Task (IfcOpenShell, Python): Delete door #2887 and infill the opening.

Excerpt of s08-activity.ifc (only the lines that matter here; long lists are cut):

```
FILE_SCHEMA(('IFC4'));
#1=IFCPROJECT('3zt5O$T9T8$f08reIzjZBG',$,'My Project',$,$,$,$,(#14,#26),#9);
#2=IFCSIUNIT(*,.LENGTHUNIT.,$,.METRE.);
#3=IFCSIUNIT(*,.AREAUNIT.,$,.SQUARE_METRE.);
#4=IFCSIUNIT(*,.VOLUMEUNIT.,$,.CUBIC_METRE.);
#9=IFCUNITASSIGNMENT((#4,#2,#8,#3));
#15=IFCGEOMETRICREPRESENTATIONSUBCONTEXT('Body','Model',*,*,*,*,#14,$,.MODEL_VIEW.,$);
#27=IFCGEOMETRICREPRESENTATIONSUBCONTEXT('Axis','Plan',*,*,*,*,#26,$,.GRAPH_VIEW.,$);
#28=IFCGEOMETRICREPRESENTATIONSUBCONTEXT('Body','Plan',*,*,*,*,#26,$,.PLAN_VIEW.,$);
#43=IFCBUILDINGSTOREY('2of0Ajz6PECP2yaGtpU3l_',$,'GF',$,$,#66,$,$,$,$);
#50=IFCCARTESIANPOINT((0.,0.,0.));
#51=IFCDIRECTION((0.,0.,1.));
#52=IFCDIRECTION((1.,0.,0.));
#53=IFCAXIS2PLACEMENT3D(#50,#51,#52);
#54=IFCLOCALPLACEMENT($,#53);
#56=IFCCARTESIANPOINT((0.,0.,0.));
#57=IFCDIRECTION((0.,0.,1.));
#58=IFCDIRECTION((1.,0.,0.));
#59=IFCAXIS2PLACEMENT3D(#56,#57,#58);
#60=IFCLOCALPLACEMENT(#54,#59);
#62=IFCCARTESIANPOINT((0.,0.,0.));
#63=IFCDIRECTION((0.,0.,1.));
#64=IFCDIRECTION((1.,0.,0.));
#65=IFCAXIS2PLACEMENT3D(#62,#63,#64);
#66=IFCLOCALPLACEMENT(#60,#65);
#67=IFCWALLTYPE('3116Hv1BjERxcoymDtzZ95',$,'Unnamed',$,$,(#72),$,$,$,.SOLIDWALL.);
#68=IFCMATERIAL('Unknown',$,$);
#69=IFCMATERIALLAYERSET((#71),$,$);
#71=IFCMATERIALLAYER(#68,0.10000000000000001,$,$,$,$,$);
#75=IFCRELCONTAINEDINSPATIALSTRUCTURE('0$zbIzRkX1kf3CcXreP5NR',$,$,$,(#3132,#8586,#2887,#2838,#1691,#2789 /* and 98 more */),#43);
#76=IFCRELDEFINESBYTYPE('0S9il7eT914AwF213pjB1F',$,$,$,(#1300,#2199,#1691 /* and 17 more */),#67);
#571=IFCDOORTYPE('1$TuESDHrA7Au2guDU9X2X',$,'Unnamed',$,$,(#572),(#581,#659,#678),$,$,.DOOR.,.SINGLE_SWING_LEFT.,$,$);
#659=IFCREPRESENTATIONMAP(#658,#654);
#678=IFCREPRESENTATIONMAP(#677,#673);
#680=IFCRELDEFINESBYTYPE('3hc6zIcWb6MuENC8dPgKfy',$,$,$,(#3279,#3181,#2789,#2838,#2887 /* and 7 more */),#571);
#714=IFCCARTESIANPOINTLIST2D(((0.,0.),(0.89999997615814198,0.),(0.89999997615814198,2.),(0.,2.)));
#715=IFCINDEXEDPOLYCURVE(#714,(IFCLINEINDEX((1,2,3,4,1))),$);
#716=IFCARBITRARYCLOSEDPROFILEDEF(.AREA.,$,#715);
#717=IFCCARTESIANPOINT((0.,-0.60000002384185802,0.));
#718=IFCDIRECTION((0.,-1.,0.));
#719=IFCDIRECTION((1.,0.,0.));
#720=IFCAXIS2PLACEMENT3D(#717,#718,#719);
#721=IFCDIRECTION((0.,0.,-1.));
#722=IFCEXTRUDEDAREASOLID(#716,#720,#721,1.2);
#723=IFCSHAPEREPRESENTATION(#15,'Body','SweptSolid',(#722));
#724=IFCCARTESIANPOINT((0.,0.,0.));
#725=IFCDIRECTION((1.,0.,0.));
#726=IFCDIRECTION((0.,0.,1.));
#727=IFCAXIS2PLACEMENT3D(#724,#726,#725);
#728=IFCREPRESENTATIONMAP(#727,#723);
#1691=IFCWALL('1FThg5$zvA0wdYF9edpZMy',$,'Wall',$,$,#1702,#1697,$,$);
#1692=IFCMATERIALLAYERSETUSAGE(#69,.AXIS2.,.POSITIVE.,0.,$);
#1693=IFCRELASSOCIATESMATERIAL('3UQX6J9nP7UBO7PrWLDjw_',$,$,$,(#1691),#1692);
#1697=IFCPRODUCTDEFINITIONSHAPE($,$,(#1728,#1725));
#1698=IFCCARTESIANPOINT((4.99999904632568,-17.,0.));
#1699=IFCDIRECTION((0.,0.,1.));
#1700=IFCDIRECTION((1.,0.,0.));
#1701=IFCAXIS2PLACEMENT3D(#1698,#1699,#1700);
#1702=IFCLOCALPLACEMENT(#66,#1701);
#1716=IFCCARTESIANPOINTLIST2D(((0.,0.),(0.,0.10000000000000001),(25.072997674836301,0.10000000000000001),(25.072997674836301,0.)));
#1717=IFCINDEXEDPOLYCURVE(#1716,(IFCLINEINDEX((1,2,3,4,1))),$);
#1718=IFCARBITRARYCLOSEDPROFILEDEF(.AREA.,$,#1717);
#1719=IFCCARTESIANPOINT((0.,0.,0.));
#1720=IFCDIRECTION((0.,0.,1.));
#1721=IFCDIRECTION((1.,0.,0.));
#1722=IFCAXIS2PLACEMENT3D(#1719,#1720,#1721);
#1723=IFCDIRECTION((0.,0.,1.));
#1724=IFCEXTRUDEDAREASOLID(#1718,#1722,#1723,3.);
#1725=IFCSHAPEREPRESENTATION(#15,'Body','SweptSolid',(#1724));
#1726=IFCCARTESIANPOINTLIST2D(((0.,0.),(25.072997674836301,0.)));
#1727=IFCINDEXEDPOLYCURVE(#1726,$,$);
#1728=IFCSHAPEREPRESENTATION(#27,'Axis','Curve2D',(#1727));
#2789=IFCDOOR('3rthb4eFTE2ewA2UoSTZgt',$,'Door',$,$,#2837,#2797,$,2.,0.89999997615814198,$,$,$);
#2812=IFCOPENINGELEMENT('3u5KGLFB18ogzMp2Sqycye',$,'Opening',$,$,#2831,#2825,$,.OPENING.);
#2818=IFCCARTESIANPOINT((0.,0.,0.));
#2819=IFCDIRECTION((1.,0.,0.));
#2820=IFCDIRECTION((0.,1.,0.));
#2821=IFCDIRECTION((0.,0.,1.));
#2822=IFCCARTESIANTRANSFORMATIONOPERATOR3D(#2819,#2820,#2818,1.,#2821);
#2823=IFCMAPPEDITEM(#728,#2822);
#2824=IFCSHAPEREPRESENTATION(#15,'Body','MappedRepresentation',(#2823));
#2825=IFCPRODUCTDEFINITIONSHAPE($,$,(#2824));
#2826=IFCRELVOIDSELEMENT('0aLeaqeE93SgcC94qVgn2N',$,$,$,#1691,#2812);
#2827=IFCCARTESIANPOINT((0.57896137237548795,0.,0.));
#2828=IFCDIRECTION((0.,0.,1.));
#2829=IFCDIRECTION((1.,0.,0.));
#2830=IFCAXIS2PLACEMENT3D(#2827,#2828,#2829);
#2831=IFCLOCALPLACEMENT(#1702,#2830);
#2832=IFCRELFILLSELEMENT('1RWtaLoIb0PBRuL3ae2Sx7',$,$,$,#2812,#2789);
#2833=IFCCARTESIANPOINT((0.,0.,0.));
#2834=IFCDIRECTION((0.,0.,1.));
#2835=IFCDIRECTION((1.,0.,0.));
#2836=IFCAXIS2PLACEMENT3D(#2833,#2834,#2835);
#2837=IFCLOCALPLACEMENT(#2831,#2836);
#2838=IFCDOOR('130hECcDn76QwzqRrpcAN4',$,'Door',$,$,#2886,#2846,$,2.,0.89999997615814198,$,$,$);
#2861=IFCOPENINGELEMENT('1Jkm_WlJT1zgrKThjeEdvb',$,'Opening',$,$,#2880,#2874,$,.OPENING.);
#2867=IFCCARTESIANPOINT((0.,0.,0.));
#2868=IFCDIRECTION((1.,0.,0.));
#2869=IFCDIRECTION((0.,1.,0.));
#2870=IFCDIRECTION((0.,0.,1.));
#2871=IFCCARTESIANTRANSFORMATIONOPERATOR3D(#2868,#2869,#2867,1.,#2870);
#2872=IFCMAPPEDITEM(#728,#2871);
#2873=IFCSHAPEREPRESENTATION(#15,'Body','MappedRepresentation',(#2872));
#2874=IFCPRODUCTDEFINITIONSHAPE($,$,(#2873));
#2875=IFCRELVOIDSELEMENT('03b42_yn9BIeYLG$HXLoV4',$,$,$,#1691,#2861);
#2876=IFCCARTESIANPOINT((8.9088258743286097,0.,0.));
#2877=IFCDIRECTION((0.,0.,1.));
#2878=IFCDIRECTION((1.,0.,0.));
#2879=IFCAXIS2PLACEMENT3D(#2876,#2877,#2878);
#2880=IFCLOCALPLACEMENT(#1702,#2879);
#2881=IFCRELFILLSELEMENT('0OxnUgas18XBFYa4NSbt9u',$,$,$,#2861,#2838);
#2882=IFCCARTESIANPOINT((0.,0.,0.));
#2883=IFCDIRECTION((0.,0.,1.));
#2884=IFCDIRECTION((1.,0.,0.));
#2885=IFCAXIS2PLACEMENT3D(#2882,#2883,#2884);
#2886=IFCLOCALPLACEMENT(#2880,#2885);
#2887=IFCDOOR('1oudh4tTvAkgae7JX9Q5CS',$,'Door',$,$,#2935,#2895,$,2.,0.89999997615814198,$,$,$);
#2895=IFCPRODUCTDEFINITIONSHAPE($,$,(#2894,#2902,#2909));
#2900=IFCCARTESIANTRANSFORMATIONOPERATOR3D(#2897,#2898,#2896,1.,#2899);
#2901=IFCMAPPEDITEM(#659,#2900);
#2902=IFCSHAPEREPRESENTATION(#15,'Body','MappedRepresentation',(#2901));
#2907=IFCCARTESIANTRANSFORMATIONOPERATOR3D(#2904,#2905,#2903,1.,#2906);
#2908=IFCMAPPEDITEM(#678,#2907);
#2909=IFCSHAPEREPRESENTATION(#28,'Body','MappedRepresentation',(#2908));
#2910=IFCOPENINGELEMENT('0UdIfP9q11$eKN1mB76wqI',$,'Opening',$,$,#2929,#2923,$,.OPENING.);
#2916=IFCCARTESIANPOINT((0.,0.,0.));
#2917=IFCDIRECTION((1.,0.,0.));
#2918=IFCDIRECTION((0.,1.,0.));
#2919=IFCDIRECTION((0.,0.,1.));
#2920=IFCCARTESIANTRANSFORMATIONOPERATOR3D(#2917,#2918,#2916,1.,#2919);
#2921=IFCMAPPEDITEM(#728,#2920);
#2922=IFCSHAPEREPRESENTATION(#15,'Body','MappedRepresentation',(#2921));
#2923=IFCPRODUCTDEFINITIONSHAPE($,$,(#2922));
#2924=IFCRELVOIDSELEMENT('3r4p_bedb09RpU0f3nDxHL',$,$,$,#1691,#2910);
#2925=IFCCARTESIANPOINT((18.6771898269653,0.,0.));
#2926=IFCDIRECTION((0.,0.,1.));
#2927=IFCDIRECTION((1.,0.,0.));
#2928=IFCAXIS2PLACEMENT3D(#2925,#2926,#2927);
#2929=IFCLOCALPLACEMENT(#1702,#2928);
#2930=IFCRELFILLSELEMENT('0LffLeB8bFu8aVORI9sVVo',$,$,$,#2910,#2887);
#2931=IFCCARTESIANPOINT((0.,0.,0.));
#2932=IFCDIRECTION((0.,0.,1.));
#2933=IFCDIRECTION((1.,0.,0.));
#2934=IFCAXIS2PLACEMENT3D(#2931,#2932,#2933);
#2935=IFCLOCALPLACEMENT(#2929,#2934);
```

```python
import ifcopenshell
import ifcopenshell.api.feature
import ifcopenshell.api.root
import ifcopenshell.geom
import ifcopenshell.util.shape

model = ifcopenshell.open("s08-activity.ifc")
settings = ifcopenshell.geom.settings()


def volume(element):
    """Net volume in cubic metres, openings subtracted."""
    shape = ifcopenshell.geom.create_shape(settings, element)
    return ifcopenshell.util.shape.get_volume(shape.geometry)


door = model.by_id(2887)
opening = door.FillsVoids[0].RelatingOpeningElement
wall = opening.VoidsElements[0].RelatingBuildingElement
before = volume(wall)

ifcopenshell.api.root.remove_product(model, product=door)
ifcopenshell.api.feature.remove_feature(model, feature=opening)

after = volume(wall)

print(f"wall volume {before:.3f} -> {after:.3f} m3")

model.write("s08-activity_rev.ifc")
```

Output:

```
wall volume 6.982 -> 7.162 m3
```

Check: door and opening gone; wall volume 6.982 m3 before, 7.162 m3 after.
